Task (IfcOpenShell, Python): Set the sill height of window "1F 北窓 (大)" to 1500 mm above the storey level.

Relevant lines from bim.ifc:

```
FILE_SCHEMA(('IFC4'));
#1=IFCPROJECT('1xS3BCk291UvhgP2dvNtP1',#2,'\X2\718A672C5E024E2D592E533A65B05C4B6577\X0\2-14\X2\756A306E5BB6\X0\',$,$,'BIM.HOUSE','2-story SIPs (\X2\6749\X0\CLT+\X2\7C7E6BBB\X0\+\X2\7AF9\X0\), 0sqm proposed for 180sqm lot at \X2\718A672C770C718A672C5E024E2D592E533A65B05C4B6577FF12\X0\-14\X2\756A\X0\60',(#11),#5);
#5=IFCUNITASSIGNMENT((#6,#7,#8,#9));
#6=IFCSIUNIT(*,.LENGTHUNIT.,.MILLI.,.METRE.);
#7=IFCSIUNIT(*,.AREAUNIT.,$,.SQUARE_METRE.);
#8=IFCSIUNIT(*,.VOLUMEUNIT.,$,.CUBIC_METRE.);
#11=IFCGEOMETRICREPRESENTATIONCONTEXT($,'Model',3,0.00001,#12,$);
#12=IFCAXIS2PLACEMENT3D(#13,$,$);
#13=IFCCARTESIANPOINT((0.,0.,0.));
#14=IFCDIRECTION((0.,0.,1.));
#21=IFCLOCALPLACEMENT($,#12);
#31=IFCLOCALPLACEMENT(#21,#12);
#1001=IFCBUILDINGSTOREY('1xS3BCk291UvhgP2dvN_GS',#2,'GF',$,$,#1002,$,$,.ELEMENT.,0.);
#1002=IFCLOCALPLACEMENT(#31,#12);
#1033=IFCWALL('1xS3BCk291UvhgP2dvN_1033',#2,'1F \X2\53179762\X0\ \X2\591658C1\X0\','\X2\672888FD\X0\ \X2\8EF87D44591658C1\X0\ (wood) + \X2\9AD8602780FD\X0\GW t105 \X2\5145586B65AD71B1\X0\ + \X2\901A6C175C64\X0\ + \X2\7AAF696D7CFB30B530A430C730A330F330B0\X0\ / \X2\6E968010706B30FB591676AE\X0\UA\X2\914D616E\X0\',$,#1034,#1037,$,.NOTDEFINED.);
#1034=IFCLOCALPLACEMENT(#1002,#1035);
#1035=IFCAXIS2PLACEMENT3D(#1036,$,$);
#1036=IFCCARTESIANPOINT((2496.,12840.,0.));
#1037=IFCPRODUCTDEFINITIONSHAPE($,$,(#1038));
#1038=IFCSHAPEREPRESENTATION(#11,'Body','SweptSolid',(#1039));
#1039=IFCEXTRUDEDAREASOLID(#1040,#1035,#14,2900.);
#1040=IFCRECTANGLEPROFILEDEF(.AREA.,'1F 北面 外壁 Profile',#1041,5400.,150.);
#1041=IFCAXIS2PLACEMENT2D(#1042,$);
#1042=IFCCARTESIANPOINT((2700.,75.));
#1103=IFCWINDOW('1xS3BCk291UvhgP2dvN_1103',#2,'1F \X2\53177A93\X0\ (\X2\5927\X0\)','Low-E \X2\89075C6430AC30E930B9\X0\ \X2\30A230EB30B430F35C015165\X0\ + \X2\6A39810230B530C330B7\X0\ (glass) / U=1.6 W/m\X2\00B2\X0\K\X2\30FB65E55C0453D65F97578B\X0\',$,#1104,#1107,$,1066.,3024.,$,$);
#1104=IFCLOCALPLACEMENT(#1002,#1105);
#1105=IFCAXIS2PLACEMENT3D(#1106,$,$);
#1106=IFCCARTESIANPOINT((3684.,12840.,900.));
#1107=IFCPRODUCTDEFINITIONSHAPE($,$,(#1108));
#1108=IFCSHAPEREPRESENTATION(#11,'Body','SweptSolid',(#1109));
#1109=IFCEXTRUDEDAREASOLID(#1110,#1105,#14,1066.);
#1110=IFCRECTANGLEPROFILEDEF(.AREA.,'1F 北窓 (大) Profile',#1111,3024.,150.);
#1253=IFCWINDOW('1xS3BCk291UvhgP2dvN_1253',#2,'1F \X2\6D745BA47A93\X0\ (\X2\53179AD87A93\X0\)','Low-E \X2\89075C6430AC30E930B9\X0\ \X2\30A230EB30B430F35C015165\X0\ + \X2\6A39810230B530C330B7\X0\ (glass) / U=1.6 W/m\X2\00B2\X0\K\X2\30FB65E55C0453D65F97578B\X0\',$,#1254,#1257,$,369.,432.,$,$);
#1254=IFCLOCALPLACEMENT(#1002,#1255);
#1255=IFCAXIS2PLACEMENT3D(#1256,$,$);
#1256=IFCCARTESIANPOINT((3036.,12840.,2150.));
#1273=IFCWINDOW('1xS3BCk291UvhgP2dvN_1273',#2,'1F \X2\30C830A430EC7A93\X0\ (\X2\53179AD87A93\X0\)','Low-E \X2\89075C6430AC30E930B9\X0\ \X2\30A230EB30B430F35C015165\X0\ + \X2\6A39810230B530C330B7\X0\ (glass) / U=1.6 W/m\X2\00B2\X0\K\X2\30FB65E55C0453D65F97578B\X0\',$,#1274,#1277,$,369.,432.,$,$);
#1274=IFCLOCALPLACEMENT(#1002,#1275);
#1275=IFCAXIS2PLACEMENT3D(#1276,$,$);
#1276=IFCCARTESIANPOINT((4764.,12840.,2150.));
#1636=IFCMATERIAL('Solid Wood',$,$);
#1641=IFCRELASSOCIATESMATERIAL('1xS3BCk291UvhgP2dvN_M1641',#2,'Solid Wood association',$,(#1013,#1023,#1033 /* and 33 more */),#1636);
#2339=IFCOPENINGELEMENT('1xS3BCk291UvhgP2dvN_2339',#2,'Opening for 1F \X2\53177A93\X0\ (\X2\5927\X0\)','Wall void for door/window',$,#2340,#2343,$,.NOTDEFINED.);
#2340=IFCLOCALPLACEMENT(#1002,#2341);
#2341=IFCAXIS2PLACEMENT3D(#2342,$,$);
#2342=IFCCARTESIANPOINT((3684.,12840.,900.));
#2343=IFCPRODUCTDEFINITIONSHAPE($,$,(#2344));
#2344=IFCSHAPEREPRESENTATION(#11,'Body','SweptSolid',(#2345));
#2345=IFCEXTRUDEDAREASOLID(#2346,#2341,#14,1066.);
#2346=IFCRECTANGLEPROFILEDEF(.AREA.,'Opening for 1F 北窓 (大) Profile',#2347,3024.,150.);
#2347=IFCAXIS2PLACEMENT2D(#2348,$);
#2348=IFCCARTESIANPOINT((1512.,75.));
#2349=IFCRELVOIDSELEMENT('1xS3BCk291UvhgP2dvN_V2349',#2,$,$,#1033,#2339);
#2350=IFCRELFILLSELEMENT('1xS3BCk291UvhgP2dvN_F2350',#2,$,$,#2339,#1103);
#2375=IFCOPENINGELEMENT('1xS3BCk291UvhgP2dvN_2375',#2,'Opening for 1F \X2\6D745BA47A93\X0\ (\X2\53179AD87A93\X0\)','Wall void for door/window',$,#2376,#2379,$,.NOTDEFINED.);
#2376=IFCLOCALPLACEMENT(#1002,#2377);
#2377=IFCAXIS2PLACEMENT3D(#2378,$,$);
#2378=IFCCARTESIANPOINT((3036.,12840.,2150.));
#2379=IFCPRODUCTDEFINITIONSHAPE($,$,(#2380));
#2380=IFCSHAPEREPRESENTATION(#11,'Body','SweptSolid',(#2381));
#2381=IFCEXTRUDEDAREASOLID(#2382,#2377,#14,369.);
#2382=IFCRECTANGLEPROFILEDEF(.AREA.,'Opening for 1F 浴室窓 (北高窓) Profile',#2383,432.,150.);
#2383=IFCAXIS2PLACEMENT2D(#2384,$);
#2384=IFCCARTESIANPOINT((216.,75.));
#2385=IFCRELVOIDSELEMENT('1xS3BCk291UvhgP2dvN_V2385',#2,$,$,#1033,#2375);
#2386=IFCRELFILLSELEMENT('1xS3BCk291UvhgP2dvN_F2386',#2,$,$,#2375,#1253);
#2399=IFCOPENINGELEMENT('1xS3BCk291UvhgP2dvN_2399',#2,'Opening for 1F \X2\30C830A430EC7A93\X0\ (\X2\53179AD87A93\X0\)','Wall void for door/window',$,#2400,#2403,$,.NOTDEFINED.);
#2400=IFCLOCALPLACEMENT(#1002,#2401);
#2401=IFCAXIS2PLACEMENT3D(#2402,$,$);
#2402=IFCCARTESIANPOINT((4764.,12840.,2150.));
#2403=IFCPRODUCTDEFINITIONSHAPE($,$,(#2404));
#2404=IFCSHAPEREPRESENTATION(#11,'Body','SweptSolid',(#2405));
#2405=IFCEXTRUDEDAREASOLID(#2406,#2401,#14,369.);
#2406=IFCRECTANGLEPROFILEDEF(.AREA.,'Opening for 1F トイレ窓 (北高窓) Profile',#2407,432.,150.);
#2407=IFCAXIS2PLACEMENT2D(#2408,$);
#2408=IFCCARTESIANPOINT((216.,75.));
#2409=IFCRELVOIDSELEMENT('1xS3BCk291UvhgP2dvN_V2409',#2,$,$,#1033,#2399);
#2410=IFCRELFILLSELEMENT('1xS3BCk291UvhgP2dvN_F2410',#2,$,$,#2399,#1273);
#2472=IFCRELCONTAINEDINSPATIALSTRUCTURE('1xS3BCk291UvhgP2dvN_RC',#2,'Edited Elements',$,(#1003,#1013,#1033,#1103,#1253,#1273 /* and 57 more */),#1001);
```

```python
import numpy as np
import ifcopenshell
import ifcopenshell.api.geometry
import ifcopenshell.geom
import ifcopenshell.util.element
import ifcopenshell.util.placement
import ifcopenshell.util.shape
import ifcopenshell.util.unit

model = ifcopenshell.open("bim.ifc")
unit_scale = ifcopenshell.util.unit.calculate_unit_scale(model)

window = model.by_guid("1xS3BCk291UvhgP2dvN_1103")
opening = window.FillsVoids[0].RelatingOpeningElement
storey = ifcopenshell.util.element.get_container(window, ifc_class="IfcBuildingStorey")
level = ifcopenshell.util.placement.get_local_placement(storey.ObjectPlacement)[2, 3]

# The opening's origin need not be at the sill, so measure its lowest point.
shape = ifcopenshell.geom.create_shape(ifcopenshell.geom.settings(), opening)
bottom = ifcopenshell.util.shape.get_shape_bottom_elevation(shape, shape.geometry) / unit_scale
dz = level + 1.5 / unit_scale - bottom

shift = np.array([0.0, 0.0, dz])
# The window is not placed relative to its opening, so move both.
for product in (opening, window):
    matrix = ifcopenshell.util.placement.get_local_placement(product.ObjectPlacement)
    matrix[:3, 3] += shift
    ifcopenshell.api.geometry.edit_object_placement(model, product=product, matrix=matrix, is_si=False)

print(f"moved by {dz * unit_scale:+.3f} m")

model.write("bim_edited.ifc")
```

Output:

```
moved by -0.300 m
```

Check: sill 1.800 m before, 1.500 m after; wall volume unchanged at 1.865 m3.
